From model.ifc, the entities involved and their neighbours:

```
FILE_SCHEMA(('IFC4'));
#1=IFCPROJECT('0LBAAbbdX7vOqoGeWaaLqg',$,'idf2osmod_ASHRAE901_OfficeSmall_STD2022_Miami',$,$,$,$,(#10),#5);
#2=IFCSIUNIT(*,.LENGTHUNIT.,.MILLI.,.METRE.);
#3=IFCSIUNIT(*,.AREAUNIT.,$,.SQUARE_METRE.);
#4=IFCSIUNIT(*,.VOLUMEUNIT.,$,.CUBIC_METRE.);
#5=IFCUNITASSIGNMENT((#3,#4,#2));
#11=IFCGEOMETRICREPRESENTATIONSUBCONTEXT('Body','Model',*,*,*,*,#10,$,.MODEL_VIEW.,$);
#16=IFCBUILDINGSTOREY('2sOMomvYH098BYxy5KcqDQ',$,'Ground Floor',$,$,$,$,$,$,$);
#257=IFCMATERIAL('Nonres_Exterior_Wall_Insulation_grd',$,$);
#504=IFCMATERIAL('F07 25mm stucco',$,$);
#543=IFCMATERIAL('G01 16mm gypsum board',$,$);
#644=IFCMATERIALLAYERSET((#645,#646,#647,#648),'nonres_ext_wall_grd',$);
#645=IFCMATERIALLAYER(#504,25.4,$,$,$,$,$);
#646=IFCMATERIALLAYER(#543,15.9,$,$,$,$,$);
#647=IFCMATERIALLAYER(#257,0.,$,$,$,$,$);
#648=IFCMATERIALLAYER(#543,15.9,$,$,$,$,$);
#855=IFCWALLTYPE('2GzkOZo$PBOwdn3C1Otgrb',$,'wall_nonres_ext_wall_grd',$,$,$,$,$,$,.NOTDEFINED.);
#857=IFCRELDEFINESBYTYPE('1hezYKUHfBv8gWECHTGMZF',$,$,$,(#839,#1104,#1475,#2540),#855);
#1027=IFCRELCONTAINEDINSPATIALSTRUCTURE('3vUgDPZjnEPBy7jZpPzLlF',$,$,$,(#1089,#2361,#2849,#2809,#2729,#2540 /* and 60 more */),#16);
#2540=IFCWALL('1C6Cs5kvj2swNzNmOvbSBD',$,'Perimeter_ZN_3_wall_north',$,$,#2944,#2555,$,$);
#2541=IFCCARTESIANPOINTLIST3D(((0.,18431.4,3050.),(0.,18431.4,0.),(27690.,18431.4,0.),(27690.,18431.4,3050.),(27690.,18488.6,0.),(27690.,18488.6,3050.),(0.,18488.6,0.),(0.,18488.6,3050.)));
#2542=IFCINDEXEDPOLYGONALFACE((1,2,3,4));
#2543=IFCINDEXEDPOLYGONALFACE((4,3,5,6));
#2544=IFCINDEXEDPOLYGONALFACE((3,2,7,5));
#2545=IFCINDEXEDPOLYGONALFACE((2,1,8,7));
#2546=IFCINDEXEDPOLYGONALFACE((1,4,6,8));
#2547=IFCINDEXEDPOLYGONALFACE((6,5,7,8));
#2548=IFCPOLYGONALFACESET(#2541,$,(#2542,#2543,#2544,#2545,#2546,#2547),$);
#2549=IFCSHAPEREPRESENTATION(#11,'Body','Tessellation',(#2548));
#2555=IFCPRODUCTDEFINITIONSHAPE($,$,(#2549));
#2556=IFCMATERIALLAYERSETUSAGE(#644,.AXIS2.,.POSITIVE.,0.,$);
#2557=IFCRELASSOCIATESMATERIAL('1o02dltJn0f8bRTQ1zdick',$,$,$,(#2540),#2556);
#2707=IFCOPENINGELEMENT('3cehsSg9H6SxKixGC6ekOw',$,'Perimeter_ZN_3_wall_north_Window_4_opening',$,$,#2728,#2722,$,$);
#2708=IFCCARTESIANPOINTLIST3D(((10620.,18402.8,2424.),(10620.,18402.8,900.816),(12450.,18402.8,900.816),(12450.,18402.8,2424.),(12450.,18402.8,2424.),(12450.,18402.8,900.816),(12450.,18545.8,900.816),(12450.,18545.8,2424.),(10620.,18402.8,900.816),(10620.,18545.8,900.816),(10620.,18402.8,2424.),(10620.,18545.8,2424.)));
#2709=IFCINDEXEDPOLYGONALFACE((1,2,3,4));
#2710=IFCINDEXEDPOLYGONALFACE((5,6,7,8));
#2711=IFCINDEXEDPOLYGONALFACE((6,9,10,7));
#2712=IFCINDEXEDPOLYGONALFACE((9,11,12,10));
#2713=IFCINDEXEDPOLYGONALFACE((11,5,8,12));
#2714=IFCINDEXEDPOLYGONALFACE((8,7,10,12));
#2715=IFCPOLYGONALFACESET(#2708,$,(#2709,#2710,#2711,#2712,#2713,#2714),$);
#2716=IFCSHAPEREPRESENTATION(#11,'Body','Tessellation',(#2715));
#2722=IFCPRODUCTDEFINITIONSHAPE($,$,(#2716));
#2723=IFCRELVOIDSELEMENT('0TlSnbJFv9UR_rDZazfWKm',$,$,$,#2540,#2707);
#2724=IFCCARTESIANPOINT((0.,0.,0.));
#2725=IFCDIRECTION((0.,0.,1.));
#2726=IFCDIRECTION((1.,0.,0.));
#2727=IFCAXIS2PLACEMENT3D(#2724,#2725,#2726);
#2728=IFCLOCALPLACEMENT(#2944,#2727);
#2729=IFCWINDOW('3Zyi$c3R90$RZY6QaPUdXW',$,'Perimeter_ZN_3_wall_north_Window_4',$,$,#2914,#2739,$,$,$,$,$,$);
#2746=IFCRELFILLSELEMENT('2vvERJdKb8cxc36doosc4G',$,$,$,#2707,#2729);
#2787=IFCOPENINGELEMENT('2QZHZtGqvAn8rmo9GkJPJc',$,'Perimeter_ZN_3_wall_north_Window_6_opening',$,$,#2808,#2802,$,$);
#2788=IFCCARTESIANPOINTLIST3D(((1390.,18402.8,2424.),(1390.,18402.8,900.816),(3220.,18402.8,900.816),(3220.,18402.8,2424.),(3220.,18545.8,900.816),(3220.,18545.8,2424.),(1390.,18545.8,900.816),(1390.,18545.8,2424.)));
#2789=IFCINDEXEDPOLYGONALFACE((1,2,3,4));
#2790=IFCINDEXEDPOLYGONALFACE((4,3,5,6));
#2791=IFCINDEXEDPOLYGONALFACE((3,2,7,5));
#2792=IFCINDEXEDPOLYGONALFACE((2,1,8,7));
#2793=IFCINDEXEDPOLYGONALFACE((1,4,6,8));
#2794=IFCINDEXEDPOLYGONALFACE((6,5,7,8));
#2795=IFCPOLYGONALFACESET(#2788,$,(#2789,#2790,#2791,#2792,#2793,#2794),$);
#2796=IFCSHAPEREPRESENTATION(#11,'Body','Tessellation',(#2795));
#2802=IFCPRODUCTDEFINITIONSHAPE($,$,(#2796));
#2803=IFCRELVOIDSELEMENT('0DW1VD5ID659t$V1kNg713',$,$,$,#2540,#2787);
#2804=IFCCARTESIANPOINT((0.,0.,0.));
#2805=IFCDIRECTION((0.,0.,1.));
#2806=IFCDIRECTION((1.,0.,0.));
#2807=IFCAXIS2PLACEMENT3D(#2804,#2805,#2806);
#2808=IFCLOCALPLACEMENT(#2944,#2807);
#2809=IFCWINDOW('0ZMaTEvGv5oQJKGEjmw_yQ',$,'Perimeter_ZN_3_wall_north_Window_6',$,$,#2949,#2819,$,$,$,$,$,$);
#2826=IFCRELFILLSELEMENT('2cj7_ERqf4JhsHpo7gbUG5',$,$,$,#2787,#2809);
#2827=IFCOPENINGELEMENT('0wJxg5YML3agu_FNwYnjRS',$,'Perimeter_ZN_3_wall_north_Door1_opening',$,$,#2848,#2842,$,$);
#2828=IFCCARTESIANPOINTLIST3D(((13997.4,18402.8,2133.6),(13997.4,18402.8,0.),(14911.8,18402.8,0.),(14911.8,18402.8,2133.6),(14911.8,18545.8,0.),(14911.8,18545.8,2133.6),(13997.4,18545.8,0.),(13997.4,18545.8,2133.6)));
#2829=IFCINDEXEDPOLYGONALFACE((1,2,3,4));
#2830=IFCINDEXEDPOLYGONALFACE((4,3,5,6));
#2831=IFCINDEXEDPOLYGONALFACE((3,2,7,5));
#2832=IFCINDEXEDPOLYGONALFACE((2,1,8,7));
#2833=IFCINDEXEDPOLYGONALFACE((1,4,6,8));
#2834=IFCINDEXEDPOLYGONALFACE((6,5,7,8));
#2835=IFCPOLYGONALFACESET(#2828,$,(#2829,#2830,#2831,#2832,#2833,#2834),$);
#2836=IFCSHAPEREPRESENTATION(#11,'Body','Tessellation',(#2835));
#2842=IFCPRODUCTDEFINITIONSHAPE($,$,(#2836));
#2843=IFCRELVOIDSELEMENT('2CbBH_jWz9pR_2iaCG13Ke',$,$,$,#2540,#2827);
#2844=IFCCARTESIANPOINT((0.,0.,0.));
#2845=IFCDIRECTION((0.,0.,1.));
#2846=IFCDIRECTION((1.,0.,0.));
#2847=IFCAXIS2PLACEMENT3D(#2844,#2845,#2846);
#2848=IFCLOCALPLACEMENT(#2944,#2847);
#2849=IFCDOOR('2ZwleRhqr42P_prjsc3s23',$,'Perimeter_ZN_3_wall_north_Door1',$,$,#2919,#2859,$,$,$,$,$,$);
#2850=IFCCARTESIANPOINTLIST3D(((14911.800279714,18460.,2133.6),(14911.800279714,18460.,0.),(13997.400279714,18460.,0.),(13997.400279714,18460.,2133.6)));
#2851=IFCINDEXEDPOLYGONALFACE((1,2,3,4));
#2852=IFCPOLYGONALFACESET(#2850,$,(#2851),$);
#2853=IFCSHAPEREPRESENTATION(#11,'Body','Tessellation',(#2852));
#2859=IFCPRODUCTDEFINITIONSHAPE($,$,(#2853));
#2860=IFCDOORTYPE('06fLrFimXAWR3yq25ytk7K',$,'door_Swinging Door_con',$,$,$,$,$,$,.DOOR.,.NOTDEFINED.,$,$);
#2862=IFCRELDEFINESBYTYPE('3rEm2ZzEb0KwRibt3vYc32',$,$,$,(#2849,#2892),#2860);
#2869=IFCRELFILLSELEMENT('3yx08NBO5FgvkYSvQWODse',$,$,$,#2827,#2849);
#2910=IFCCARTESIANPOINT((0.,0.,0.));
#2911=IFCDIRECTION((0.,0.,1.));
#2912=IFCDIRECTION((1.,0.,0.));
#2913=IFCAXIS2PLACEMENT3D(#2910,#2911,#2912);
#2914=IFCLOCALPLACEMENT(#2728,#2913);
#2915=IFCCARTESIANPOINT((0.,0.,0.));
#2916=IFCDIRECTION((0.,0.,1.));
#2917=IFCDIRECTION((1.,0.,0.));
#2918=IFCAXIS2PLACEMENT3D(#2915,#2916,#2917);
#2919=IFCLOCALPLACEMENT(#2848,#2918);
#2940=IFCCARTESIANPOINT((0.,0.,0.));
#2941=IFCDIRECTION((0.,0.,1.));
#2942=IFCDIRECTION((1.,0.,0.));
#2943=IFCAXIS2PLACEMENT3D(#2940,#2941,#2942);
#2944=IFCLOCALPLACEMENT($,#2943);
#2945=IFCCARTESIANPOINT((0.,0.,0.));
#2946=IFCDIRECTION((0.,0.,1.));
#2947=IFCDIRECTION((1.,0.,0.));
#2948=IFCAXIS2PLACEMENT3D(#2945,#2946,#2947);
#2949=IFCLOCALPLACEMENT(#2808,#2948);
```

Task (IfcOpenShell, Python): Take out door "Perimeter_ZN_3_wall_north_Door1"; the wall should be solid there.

```python
import ifcopenshell
import ifcopenshell.api.feature
import ifcopenshell.api.root
import ifcopenshell.geom
import ifcopenshell.util.shape

model = ifcopenshell.open("model.ifc")
settings = ifcopenshell.geom.settings()


def volume(element):
    """Net volume in cubic metres, openings subtracted."""
    shape = ifcopenshell.geom.create_shape(settings, element)
    return ifcopenshell.util.shape.get_volume(shape.geometry)


door = model.by_guid("2ZwleRhqr42P_prjsc3s23")
opening = door.FillsVoids[0].RelatingOpeningElement
wall = opening.VoidsElements[0].RelatingBuildingElement
before = volume(wall)

ifcopenshell.api.root.remove_product(model, product=door)
ifcopenshell.api.feature.remove_feature(model, feature=opening)

after = volume(wall)

print(f"wall volume {before:.3f} -> {after:.3f} m3")

model.write("model-out.ifc")
```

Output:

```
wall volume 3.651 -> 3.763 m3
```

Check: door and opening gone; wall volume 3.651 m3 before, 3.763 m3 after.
